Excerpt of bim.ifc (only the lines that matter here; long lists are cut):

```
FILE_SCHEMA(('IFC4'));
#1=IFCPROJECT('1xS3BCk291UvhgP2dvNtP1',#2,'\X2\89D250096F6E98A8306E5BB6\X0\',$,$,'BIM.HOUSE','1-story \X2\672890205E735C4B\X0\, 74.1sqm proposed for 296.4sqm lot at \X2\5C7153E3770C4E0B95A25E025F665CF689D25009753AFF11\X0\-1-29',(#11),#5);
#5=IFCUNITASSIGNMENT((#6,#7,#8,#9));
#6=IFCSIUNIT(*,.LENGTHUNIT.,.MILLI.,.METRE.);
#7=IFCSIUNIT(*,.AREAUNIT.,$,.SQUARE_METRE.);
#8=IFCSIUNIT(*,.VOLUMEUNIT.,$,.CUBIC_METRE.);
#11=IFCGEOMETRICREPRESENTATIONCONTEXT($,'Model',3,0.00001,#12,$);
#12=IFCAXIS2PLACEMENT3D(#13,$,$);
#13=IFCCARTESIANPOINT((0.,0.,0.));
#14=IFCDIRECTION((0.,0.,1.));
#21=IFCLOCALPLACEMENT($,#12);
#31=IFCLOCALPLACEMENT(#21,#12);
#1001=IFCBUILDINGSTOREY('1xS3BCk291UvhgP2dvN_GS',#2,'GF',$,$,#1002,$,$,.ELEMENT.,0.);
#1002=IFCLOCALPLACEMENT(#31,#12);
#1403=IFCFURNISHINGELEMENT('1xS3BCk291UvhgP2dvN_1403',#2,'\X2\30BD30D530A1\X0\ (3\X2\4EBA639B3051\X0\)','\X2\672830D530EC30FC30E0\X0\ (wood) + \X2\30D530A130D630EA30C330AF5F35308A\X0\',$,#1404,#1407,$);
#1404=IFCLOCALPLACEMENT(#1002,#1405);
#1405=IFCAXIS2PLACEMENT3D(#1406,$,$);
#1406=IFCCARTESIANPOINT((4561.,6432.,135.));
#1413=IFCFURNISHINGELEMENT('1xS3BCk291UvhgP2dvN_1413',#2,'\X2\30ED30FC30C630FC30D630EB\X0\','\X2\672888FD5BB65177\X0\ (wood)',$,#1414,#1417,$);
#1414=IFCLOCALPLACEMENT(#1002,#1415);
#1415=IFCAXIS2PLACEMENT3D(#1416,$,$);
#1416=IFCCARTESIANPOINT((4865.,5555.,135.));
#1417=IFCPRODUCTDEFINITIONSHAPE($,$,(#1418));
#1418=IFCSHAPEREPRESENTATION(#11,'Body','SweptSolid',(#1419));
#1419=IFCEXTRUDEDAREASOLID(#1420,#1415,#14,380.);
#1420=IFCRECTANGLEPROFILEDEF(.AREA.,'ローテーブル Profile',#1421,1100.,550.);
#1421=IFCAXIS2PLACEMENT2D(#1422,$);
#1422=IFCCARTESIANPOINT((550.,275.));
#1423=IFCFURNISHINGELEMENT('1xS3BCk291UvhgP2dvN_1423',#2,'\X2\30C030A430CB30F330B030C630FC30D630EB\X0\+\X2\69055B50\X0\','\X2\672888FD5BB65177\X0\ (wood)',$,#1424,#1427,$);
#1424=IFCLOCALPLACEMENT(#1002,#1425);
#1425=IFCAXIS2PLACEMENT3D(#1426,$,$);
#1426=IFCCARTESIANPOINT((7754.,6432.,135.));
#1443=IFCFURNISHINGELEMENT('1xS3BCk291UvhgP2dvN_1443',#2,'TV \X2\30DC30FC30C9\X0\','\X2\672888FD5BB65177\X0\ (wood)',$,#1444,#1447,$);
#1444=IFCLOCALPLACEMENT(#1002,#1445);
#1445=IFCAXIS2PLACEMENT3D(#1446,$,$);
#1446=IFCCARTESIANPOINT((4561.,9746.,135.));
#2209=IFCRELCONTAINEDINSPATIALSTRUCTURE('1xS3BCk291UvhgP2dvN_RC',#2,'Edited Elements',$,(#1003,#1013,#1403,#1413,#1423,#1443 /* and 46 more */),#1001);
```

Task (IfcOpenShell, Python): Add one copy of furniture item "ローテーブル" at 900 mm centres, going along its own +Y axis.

```python
import ifcopenshell
import ifcopenshell.api.geometry
import ifcopenshell.api.root
import ifcopenshell.util.element
import ifcopenshell.util.placement
import ifcopenshell.util.unit

model = ifcopenshell.open("bim.ifc")
unit_scale = ifcopenshell.util.unit.calculate_unit_scale(model)


def reuse_history(source, copy):
    """copy_class also copies each property set's owner history, people and application; keep the originals."""
    for rel in copy.IsDefinedBy:
        if rel.is_a("IfcRelDefinesByProperties") and (history := rel.RelatingPropertyDefinition.OwnerHistory):
            rel.RelatingPropertyDefinition.OwnerHistory = source.OwnerHistory
            ifcopenshell.util.element.remove_deep2(model, history)


source = model.by_guid("1xS3BCk291UvhgP2dvN_1413")
base = ifcopenshell.util.placement.get_local_placement(source.ObjectPlacement)
step = base[:3, 1] * 0.9 / unit_scale

for i in range(1, 2):
    copy = ifcopenshell.api.root.copy_class(model, product=source)
    copy.Representation = ifcopenshell.util.element.copy_deep(
        model, source.Representation, exclude=["IfcGeometricRepresentationContext", "IfcRepresentationMap"]
    )
    reuse_history(source, copy)
    matrix = base.copy()
    matrix[:3, 3] += i * step
    print("added at", matrix[:3, 3].round(3) + 0.0)
    ifcopenshell.api.geometry.edit_object_placement(model, product=copy, matrix=matrix, is_si=False)

model.write("bim_updated.ifc")
```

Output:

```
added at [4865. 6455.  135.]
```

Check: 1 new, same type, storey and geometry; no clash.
